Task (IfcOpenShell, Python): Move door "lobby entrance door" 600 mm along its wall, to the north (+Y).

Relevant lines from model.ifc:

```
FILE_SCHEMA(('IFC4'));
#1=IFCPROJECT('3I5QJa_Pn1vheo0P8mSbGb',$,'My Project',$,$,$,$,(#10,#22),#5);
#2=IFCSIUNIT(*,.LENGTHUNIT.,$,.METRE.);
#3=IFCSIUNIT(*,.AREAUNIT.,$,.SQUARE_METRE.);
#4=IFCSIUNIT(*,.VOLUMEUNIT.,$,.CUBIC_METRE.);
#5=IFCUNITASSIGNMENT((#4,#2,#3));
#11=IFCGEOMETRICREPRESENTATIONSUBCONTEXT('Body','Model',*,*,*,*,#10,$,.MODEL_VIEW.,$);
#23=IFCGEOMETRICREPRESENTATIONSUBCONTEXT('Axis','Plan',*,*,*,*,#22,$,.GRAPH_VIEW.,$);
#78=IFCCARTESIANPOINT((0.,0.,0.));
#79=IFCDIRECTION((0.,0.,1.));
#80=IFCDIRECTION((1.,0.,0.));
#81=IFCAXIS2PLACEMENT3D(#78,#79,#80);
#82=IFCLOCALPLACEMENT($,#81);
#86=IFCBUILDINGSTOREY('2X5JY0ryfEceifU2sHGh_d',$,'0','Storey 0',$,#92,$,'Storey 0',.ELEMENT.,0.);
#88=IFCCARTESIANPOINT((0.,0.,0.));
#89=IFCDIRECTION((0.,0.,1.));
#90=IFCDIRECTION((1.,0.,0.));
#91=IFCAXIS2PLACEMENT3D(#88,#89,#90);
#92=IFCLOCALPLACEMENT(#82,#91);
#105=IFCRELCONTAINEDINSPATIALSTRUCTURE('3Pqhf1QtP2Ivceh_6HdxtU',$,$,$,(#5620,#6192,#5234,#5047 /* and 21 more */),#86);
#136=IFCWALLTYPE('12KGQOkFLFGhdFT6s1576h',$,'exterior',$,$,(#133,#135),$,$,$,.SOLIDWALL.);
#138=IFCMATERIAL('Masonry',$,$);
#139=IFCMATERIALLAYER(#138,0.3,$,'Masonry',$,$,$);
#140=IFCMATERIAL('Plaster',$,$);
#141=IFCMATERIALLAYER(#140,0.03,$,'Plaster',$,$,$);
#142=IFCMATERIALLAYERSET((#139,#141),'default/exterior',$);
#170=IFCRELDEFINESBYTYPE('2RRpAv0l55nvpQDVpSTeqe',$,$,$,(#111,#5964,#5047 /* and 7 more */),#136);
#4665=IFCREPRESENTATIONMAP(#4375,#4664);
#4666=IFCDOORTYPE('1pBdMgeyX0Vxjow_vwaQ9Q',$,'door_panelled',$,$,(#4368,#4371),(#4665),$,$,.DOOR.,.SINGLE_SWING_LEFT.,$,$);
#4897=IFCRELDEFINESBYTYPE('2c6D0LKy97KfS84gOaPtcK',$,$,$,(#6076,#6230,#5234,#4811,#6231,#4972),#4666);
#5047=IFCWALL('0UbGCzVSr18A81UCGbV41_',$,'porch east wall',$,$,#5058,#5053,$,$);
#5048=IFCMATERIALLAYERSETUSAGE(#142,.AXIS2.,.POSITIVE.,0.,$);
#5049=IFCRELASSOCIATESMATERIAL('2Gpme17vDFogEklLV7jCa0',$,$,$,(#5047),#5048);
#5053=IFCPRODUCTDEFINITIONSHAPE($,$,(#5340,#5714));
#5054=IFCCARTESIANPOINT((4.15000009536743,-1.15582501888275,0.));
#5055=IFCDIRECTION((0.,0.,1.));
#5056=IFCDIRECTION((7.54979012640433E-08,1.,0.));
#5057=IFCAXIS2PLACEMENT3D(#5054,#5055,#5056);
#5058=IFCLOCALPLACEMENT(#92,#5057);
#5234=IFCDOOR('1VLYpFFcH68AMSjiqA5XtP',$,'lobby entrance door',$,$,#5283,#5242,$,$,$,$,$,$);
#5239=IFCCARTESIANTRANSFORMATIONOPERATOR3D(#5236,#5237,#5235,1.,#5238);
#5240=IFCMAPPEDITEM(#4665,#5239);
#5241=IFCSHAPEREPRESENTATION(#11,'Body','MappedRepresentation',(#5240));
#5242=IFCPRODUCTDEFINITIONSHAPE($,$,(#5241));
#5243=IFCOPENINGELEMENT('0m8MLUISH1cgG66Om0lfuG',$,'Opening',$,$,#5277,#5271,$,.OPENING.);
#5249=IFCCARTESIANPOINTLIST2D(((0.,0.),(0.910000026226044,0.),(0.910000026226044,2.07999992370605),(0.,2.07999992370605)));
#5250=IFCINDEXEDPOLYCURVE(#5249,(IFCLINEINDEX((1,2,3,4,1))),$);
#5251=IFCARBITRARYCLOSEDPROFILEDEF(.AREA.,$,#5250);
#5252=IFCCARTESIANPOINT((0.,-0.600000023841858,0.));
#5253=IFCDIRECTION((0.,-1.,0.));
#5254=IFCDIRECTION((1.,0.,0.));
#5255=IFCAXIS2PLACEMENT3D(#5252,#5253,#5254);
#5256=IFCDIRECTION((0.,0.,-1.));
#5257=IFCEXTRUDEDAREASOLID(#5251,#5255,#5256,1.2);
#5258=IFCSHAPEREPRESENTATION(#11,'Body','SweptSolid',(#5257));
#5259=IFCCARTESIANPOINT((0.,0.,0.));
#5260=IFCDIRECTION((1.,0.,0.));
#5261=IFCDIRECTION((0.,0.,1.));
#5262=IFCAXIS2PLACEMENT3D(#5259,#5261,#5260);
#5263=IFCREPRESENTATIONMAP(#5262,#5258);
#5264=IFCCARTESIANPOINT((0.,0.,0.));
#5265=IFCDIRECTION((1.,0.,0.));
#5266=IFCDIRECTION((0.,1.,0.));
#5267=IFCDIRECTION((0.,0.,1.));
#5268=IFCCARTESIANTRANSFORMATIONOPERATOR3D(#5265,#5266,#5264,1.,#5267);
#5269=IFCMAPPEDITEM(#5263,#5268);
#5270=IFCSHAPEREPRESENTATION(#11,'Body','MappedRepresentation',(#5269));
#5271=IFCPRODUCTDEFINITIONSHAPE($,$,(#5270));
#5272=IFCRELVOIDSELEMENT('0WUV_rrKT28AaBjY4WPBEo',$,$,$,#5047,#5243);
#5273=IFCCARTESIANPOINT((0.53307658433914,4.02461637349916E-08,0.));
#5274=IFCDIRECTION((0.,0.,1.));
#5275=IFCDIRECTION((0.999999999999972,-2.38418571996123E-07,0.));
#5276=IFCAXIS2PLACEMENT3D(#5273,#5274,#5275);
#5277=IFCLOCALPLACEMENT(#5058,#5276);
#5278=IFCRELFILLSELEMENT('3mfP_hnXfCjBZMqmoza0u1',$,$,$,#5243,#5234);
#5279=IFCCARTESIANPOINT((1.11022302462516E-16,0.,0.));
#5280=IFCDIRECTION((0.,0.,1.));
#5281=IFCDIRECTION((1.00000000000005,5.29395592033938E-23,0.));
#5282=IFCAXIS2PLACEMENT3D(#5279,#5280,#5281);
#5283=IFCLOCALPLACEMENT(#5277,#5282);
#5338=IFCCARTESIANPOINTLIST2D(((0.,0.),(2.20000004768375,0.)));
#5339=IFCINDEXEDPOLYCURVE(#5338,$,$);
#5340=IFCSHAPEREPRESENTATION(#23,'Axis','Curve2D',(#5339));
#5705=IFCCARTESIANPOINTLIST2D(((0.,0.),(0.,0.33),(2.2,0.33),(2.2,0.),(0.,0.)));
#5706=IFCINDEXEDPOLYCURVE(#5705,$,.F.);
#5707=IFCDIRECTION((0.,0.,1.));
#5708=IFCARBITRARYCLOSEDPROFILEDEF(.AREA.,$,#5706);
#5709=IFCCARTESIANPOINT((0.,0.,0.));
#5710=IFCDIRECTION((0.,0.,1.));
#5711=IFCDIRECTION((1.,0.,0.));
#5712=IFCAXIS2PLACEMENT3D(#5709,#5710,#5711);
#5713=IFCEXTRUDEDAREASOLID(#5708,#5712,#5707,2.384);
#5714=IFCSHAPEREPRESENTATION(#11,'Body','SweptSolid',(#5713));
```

```python
import ifcopenshell
import ifcopenshell.api.geometry
import ifcopenshell.util.placement
import ifcopenshell.util.unit

model = ifcopenshell.open("model.ifc")
unit_scale = ifcopenshell.util.unit.calculate_unit_scale(model)

door = model.by_guid("1VLYpFFcH68AMSjiqA5XtP")
opening = door.FillsVoids[0].RelatingOpeningElement
wall = opening.VoidsElements[0].RelatingBuildingElement

wall_matrix = ifcopenshell.util.placement.get_local_placement(wall.ObjectPlacement)
shift = wall_matrix[:3, 0] * 0.6 / unit_scale
before = ifcopenshell.util.placement.get_local_placement(door.ObjectPlacement)[:3, 3].copy()

# The door is placed relative to its opening, so it follows when the opening moves.
matrix = ifcopenshell.util.placement.get_local_placement(opening.ObjectPlacement)
matrix[:3, 3] += shift
ifcopenshell.api.geometry.edit_object_placement(
    model, product=opening, matrix=matrix, is_si=False, should_transform_children=True
)

after = ifcopenshell.util.placement.get_local_placement(door.ObjectPlacement)[:3, 3]
print("door moved by", (after - before).round(3) + 0.0)

model.write("model_updated.ifc")
```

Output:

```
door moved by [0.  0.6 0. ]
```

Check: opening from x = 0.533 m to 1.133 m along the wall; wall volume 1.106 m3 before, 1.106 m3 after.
